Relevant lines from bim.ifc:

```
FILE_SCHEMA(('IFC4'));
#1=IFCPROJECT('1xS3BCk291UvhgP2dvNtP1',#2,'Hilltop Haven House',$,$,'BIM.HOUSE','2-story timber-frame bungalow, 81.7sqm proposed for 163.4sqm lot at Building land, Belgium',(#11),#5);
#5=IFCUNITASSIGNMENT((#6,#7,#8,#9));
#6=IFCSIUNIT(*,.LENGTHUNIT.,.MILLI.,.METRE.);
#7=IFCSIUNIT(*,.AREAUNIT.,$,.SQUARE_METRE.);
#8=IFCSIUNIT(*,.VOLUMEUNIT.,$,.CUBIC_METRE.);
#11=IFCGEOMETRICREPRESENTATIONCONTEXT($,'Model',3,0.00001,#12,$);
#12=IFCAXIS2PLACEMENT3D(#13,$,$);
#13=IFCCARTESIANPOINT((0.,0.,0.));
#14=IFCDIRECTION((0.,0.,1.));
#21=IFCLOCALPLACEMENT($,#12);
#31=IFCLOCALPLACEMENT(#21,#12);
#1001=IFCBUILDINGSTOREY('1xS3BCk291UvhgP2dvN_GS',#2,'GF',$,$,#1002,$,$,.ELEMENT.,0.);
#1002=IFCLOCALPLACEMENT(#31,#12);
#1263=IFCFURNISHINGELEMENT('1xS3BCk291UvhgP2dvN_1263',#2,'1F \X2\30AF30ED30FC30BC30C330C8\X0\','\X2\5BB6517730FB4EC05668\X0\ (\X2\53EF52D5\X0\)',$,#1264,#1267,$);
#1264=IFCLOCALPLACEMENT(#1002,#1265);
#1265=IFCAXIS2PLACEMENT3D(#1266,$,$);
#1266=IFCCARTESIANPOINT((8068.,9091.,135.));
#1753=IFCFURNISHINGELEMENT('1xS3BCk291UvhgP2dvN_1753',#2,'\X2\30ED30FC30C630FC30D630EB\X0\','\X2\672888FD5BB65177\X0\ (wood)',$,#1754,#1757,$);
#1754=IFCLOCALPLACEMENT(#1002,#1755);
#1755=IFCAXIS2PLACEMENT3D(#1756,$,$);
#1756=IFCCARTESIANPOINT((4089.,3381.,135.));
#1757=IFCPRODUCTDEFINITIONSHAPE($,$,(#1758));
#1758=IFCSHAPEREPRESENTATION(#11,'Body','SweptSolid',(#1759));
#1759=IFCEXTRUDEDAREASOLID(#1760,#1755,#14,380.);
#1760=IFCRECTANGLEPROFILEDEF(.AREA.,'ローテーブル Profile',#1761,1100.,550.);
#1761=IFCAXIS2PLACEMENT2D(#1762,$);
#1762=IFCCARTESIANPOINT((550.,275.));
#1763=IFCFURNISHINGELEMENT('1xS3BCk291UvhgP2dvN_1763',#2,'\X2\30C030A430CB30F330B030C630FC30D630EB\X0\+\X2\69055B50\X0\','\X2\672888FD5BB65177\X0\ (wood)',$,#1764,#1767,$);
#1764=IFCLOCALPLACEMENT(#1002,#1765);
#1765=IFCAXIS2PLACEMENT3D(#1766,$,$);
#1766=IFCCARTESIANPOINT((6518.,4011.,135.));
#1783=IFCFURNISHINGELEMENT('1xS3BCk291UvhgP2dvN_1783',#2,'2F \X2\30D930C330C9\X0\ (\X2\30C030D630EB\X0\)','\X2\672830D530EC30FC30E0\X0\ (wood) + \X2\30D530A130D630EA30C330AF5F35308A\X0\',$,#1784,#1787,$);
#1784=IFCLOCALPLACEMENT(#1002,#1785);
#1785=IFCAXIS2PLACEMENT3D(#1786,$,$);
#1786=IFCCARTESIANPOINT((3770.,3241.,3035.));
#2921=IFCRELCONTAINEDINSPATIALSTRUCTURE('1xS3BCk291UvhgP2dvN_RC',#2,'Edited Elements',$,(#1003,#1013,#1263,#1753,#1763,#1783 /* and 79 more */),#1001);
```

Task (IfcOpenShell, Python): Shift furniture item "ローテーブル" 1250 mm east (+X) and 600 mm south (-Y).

```python
import ifcopenshell
import ifcopenshell.api.geometry
import ifcopenshell.util.placement
import ifcopenshell.util.unit

model = ifcopenshell.open("bim.ifc")
unit_scale = ifcopenshell.util.unit.calculate_unit_scale(model)

item = model.by_guid("1xS3BCk291UvhgP2dvN_1753")
matrix = ifcopenshell.util.placement.get_local_placement(item.ObjectPlacement)
matrix[0, 3] += 1.25 / unit_scale
matrix[1, 3] -= 0.6 / unit_scale
ifcopenshell.api.geometry.edit_object_placement(model, product=item, matrix=matrix, is_si=False)

print(ifcopenshell.util.placement.get_local_placement(item.ObjectPlacement).round(3) + 0.0)

model.write("bim_v2.ifc")
```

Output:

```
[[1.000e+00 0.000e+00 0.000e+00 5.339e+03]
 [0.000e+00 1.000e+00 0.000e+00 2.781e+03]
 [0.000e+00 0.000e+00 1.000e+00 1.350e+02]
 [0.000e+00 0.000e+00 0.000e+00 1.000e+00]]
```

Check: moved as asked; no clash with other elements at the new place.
